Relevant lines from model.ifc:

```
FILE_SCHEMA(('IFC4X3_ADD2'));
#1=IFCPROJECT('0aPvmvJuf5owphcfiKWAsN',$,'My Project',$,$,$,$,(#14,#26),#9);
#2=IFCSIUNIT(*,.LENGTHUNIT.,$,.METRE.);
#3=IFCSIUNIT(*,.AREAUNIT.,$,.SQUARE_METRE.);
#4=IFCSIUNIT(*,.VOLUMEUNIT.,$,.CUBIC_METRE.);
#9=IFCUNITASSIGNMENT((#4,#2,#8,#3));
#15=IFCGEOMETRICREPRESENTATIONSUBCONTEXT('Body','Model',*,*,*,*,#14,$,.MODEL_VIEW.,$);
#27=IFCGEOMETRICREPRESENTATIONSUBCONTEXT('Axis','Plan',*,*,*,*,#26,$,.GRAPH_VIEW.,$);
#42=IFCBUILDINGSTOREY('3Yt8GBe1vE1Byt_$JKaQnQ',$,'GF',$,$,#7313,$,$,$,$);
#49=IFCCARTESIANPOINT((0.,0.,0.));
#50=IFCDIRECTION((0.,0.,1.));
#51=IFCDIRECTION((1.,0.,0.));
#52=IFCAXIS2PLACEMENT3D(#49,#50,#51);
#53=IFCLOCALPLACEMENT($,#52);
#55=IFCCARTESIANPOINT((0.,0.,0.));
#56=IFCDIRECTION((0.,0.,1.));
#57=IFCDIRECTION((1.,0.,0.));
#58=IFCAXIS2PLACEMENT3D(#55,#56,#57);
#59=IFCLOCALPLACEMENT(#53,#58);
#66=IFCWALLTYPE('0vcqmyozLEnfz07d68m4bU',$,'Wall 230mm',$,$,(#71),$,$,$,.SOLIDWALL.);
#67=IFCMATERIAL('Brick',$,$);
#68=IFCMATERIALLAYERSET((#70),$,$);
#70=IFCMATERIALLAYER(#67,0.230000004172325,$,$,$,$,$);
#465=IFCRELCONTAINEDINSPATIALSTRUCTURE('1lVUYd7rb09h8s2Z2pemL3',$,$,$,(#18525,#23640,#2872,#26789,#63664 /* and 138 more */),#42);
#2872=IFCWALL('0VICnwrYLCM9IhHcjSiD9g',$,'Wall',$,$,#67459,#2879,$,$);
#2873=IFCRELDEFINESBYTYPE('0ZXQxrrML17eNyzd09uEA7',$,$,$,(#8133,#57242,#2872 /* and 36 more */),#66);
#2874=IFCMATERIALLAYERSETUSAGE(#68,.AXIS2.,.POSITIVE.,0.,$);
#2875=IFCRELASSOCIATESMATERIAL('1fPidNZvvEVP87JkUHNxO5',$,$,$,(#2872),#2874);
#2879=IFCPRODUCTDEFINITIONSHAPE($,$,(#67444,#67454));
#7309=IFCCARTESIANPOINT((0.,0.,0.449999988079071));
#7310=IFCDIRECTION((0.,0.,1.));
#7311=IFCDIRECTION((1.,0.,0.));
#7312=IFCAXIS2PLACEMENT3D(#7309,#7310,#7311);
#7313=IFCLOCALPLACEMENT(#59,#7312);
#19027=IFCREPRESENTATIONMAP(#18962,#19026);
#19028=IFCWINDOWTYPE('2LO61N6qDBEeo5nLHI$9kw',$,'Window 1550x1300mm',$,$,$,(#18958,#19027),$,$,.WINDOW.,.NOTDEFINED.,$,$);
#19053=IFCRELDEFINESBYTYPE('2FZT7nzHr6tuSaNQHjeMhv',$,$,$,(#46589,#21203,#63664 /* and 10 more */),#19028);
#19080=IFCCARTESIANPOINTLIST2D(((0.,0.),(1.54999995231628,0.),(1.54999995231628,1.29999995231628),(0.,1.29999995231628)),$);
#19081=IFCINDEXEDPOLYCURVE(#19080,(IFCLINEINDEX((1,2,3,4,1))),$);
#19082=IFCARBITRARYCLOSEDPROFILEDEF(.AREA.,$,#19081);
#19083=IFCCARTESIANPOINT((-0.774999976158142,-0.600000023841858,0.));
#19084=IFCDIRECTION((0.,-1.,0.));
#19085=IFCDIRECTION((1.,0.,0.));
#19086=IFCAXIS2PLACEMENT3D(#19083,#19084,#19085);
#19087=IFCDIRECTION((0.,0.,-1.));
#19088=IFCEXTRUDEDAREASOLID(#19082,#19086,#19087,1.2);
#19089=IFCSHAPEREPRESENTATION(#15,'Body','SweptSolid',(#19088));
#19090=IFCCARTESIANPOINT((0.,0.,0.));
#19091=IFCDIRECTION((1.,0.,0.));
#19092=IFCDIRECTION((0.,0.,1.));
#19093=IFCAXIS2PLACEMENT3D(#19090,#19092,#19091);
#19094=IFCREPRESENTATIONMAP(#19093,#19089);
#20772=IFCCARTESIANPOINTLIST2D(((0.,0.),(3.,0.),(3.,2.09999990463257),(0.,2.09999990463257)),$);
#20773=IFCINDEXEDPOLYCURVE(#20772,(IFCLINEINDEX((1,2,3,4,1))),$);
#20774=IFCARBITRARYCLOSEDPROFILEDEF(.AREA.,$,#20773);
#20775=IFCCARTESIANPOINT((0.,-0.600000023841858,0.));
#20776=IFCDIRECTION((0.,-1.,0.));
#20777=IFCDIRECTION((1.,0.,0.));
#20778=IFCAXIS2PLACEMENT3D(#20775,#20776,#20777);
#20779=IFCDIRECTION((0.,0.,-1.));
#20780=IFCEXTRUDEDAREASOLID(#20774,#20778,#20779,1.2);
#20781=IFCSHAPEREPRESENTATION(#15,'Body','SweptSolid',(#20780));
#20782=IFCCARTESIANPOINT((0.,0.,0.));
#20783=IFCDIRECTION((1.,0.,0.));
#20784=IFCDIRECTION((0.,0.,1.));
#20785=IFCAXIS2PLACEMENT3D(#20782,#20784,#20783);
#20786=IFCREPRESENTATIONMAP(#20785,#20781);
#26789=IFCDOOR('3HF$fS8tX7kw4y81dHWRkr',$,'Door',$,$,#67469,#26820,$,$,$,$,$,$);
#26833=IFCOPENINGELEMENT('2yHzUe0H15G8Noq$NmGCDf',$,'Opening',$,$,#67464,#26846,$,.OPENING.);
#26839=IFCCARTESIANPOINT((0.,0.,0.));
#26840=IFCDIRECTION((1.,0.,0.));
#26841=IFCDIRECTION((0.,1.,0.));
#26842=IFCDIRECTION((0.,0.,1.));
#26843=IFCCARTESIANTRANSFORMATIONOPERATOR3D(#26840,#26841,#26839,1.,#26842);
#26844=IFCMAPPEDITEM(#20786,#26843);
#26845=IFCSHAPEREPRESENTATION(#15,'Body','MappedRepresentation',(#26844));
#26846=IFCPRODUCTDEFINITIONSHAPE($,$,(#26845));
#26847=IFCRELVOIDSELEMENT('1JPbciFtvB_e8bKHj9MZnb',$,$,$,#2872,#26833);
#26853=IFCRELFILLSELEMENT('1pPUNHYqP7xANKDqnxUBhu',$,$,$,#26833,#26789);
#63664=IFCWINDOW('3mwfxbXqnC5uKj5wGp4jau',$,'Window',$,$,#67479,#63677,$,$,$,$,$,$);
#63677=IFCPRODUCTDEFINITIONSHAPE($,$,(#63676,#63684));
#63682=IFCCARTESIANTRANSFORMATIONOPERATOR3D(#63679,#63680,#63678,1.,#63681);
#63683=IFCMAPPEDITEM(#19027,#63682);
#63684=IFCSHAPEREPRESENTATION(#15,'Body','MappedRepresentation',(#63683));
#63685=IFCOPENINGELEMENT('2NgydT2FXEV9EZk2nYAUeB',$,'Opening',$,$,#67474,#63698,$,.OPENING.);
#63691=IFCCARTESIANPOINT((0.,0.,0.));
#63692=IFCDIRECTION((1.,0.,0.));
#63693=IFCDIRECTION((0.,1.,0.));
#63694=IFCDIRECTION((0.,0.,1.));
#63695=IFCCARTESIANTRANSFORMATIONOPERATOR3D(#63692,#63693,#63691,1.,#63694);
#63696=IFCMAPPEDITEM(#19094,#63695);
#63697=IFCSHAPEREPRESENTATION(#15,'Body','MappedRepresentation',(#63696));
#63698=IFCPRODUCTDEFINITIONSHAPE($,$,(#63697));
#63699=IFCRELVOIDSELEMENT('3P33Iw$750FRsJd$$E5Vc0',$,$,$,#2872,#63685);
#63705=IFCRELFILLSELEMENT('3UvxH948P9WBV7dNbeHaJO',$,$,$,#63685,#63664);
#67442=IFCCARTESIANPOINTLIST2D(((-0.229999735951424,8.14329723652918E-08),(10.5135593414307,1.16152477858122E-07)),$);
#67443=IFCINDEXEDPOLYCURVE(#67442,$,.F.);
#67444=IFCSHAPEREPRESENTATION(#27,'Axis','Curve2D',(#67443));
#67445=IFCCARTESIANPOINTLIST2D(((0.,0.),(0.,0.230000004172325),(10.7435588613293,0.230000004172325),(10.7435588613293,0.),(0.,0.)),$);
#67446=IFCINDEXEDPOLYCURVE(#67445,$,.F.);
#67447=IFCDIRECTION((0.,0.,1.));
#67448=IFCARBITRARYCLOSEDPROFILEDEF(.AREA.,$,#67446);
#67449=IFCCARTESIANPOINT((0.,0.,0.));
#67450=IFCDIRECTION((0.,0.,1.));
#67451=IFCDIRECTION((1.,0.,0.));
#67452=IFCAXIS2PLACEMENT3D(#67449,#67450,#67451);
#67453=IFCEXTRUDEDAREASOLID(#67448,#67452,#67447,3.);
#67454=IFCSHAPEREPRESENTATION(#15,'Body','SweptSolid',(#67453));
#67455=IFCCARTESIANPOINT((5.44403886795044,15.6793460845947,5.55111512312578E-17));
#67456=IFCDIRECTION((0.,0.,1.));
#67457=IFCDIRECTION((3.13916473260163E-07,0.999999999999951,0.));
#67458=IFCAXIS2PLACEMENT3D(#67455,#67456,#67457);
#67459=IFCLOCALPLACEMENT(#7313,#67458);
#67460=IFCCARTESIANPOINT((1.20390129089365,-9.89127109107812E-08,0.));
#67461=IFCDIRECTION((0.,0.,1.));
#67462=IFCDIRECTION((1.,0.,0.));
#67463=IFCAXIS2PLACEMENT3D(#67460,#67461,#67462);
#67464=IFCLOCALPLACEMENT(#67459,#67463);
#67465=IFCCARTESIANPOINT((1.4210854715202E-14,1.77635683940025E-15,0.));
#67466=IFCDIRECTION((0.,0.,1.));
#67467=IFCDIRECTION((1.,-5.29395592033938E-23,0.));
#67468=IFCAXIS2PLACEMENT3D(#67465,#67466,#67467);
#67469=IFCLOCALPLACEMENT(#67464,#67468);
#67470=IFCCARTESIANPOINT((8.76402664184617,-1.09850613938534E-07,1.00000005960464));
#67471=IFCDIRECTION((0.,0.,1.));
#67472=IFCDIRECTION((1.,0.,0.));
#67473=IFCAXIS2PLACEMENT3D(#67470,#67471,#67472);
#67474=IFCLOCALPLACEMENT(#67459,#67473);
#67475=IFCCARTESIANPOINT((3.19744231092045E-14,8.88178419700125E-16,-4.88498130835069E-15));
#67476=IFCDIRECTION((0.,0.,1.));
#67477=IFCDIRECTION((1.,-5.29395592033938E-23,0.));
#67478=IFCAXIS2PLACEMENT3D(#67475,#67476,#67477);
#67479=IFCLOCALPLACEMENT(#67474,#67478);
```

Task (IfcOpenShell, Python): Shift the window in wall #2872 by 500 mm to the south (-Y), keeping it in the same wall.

```python
import ifcopenshell
import ifcopenshell.api.geometry
import ifcopenshell.util.placement
import ifcopenshell.util.unit

model = ifcopenshell.open("model.ifc")
unit_scale = ifcopenshell.util.unit.calculate_unit_scale(model)

window = model.by_guid("3mwfxbXqnC5uKj5wGp4jau")
opening = window.FillsVoids[0].RelatingOpeningElement
wall = opening.VoidsElements[0].RelatingBuildingElement

wall_matrix = ifcopenshell.util.placement.get_local_placement(wall.ObjectPlacement)
shift = wall_matrix[:3, 0] * -0.5 / unit_scale
before = ifcopenshell.util.placement.get_local_placement(window.ObjectPlacement)[:3, 3].copy()

# The window is placed relative to its opening, so it follows when the opening moves.
matrix = ifcopenshell.util.placement.get_local_placement(opening.ObjectPlacement)
matrix[:3, 3] += shift
ifcopenshell.api.geometry.edit_object_placement(
    model, product=opening, matrix=matrix, is_si=False, should_transform_children=True
)

after = ifcopenshell.util.placement.get_local_placement(window.ObjectPlacement)[:3, 3]
print("window moved by", (after - before).round(3) + 0.0)

model.write("model_updated.ifc")
```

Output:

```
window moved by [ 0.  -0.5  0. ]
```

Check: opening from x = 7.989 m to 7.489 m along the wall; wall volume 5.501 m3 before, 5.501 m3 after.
